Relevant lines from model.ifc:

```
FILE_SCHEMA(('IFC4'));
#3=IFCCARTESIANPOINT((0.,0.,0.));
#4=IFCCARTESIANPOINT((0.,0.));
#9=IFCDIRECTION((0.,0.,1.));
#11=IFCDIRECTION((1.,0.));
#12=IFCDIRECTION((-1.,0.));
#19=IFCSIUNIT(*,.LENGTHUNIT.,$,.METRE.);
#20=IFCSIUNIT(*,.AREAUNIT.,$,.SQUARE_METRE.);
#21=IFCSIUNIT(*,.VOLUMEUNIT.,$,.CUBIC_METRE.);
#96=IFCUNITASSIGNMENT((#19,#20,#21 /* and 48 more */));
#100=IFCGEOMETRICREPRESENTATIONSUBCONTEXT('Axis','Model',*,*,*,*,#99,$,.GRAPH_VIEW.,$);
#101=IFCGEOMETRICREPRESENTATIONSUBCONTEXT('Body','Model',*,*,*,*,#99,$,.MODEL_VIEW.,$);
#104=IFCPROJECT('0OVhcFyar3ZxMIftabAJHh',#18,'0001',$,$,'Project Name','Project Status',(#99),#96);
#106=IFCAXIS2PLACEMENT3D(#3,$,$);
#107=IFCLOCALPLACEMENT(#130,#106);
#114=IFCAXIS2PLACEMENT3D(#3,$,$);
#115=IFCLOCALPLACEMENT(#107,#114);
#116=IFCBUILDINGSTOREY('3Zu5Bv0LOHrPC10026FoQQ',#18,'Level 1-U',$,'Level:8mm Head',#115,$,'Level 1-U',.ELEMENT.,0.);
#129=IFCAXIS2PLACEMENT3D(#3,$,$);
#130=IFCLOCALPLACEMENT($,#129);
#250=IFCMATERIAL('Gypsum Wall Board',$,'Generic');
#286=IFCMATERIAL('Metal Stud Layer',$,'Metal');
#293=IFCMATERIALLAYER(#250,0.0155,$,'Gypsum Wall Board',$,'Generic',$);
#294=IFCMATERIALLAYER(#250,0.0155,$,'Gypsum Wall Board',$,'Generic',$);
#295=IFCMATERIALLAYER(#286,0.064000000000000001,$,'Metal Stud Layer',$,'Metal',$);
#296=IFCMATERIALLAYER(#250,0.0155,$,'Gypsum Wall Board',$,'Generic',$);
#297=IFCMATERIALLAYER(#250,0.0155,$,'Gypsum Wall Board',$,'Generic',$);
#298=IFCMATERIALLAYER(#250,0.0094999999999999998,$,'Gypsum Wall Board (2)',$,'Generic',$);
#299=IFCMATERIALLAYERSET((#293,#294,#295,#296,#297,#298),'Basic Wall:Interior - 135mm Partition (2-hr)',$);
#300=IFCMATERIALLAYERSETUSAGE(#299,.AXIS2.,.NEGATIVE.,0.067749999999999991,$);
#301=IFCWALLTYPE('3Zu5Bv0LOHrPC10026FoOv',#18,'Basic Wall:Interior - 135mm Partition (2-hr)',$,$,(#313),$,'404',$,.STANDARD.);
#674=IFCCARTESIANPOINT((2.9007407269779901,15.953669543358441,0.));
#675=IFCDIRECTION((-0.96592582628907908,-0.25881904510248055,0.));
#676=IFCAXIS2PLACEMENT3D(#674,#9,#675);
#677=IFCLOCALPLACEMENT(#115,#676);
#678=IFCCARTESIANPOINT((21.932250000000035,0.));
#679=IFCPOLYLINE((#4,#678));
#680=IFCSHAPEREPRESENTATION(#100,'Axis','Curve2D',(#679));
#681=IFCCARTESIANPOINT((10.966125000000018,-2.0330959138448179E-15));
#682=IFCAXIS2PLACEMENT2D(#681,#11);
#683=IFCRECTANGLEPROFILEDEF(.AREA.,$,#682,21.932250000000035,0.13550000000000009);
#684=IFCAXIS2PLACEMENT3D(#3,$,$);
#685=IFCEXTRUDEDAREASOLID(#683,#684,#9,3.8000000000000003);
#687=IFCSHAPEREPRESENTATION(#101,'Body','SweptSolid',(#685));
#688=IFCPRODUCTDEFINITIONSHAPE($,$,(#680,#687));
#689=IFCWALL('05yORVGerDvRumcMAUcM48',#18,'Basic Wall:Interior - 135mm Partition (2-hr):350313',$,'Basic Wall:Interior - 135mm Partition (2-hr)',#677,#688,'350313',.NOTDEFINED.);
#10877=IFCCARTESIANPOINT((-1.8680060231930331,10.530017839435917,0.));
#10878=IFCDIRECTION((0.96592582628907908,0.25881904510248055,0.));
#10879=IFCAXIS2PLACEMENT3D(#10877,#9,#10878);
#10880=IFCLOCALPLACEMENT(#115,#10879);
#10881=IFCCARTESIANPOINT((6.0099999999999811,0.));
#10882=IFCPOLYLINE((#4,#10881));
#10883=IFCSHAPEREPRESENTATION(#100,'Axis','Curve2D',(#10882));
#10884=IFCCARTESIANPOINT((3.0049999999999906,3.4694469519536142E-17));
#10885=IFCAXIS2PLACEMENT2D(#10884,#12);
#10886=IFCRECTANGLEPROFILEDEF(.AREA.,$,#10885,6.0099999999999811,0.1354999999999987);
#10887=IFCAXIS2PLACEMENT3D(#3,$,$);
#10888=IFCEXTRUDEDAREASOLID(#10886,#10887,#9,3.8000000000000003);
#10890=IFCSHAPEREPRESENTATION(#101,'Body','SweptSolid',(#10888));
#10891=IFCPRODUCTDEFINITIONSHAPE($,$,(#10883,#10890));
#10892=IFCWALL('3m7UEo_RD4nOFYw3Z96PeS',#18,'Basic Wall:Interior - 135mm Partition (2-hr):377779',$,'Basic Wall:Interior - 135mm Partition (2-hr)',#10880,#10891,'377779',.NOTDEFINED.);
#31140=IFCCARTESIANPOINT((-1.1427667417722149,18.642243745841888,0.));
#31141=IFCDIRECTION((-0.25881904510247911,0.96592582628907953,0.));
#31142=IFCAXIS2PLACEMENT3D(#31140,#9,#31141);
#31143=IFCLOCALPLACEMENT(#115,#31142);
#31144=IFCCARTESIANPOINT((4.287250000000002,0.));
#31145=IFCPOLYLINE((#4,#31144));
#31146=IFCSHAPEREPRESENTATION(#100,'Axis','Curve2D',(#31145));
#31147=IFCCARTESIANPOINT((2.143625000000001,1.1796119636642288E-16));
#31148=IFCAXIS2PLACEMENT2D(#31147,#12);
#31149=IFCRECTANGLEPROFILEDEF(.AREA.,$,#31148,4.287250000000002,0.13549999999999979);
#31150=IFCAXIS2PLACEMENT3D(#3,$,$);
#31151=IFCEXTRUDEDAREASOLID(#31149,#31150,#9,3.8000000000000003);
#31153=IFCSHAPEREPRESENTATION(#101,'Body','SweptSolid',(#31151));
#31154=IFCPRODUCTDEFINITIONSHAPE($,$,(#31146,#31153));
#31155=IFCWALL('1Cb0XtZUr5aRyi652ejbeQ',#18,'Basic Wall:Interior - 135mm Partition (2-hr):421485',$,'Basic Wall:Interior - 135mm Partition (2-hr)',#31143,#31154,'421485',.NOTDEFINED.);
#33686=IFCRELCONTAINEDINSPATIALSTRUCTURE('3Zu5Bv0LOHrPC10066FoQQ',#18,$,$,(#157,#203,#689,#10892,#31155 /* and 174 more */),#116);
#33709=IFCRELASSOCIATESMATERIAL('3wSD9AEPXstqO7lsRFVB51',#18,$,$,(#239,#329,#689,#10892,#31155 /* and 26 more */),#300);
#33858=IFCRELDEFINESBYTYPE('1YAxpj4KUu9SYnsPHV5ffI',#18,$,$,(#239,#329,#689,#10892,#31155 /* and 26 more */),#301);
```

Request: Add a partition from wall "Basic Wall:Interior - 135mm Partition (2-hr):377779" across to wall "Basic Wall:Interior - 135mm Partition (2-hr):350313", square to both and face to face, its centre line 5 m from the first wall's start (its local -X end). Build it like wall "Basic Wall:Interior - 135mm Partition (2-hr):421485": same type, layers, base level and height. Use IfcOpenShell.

```python
import numpy as np
import ifcopenshell
import ifcopenshell.api.geometry
import ifcopenshell.api.material
import ifcopenshell.api.pset
import ifcopenshell.api.root
import ifcopenshell.api.spatial
import ifcopenshell.api.type
import ifcopenshell.geom
import ifcopenshell.util.element
import ifcopenshell.util.placement
import ifcopenshell.util.representation
import ifcopenshell.util.shape
import ifcopenshell.util.unit

model = ifcopenshell.open("model.ifc")
unit_scale = ifcopenshell.util.unit.calculate_unit_scale(model)
settings = ifcopenshell.geom.settings()
settings.set("use-world-coords", True)

start_wall = model.by_id(10892)
end_wall = model.by_id(689)
like = model.by_guid("1Cb0XtZUr5aRyi652ejbeQ")
matrix = ifcopenshell.util.placement.get_local_placement(start_wall.ObjectPlacement)
matrix[:3, 3] *= unit_scale


def extent(element):
    """Bounding box in the first wall's axes, in metres."""
    shape = ifcopenshell.geom.create_shape(settings, element)
    points = (ifcopenshell.util.shape.get_vertices(shape.geometry) - matrix[:3, 3]) @ matrix[:3, :3]
    return points.min(axis=0), points.max(axis=0)


y_start = extent(start_wall)[1][1]
y_end = extent(end_wall)[0][1]
like_min, like_max = extent(like)
length, height = float(abs(y_end - y_start)), float(like_max[2] - like_min[2])
layer_set = ifcopenshell.util.element.get_material(like, should_skip_usage=True)
thickness = sum(layer.LayerThickness for layer in layer_set.MaterialLayers) * unit_scale

wall = ifcopenshell.api.root.create_entity(model, ifc_class="IfcWall", name="New partition")
storey = ifcopenshell.util.element.get_container(like)
ifcopenshell.api.spatial.assign_container(model, products=[wall], relating_structure=storey)
ifcopenshell.api.type.assign_type(
    model, related_objects=[wall], relating_type=ifcopenshell.util.element.get_type(like), should_map_representations=False
)
rel = ifcopenshell.api.material.assign_material(
    model, products=[wall], type="IfcMaterialLayerSetUsage", material=layer_set
)
rel.RelatingMaterial.OffsetFromReferenceLine = -thickness / 2 / unit_scale
pset = ifcopenshell.api.pset.add_pset(model, product=wall, name="Pset_WallCommon")
ifcopenshell.api.pset.edit_pset(model, pset=pset, properties={"IsExternal": False, "LoadBearing": False})

# The axis runs down the middle of the wall.
axis = ifcopenshell.api.geometry.add_axis_representation(
    model, context=ifcopenshell.util.representation.get_context(model, "Model", "Axis"), axis=[(0.0, 0.0), (length, 0.0)]
)
body = ifcopenshell.api.geometry.add_wall_representation(
    model,
    context=ifcopenshell.util.representation.get_context(model, "Model", "Body", "MODEL_VIEW"),
    length=length,
    height=height,
    thickness=thickness,
    offset=-thickness / 2,
)
for representation in (axis, body):
    ifcopenshell.api.geometry.assign_representation(model, product=wall, representation=representation)

placement = matrix @ ifcopenshell.util.placement.rotation(90, "Z")
placement[:, 3] = matrix @ np.array([extent(start_wall)[0][0] + 5, y_start, like_min[2], 1.0])
ifcopenshell.api.geometry.edit_object_placement(model, product=wall, matrix=placement)

print(f"partition {length:.3f} m long, {height:.3f} m high, {thickness:.3f} m thick")

model.write("model_v2.ifc")
```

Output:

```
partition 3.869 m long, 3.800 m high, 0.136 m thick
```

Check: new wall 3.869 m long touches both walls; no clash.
